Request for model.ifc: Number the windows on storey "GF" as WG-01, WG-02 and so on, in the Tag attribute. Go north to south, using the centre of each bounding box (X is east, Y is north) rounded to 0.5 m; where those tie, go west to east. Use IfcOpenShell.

First a look at what the model holds.

```python
import ifcopenshell
import ifcopenshell.util.element
import ifcopenshell.util.placement

model = ifcopenshell.open("model.ifc")
print(model.schema)
storey = next(s for s in model.by_type("IfcBuildingStorey") if s.Name == "GF")
windows = [e for e in ifcopenshell.util.element.get_decomposition(storey) if e.is_a("IfcWindow")]
for e in sorted(windows, key=lambda e: e.id()):
    origin = ifcopenshell.util.placement.get_local_placement(e.ObjectPlacement)[:3, 3]
    print(e.id(), e.Tag, e.Name, origin.round(2) + 0.0, sep=" | ")
```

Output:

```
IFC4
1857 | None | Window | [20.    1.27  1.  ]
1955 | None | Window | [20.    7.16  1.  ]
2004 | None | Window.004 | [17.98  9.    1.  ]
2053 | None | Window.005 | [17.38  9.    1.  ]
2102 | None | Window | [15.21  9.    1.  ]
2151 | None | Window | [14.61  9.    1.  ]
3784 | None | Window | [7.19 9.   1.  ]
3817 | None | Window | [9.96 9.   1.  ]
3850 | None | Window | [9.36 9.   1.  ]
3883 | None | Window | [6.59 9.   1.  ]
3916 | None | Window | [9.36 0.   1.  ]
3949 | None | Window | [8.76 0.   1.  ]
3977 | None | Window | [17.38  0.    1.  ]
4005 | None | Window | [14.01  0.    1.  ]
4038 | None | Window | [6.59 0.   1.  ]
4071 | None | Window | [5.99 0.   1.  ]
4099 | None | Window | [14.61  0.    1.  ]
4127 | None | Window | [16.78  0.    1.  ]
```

```python
import ifcopenshell
import ifcopenshell.geom
import ifcopenshell.util.element
import ifcopenshell.util.shape

model = ifcopenshell.open("model.ifc")
settings = ifcopenshell.geom.settings()
settings.set("use-world-coords", True)


def centre(element):
    shape = ifcopenshell.geom.create_shape(settings, element)
    return ifcopenshell.util.shape.get_bbox_centroid(shape.geometry)


storey = next(s for s in model.by_type("IfcBuildingStorey") if s.Name == "GF")
windows = [e for e in ifcopenshell.util.element.get_decomposition(storey) if e.is_a("IfcWindow")]

# Insertion points can sit at a corner or the storey origin, so sort by the geometry (in metres).
centres = {e: centre(e) for e in windows}
windows.sort(key=lambda e: (-round(centres[e][1] / 0.5), centres[e][0]))

for i, e in enumerate(windows, start=1):
    number = f"WG-{i:02d}"
    e.Tag = number
    print(e.id(), number)

model.write("model_rev.ifc")
```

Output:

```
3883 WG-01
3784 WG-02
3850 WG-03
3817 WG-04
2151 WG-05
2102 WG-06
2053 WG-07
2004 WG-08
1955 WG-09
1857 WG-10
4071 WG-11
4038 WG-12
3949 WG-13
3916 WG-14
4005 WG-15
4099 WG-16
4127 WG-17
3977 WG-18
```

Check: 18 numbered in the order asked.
